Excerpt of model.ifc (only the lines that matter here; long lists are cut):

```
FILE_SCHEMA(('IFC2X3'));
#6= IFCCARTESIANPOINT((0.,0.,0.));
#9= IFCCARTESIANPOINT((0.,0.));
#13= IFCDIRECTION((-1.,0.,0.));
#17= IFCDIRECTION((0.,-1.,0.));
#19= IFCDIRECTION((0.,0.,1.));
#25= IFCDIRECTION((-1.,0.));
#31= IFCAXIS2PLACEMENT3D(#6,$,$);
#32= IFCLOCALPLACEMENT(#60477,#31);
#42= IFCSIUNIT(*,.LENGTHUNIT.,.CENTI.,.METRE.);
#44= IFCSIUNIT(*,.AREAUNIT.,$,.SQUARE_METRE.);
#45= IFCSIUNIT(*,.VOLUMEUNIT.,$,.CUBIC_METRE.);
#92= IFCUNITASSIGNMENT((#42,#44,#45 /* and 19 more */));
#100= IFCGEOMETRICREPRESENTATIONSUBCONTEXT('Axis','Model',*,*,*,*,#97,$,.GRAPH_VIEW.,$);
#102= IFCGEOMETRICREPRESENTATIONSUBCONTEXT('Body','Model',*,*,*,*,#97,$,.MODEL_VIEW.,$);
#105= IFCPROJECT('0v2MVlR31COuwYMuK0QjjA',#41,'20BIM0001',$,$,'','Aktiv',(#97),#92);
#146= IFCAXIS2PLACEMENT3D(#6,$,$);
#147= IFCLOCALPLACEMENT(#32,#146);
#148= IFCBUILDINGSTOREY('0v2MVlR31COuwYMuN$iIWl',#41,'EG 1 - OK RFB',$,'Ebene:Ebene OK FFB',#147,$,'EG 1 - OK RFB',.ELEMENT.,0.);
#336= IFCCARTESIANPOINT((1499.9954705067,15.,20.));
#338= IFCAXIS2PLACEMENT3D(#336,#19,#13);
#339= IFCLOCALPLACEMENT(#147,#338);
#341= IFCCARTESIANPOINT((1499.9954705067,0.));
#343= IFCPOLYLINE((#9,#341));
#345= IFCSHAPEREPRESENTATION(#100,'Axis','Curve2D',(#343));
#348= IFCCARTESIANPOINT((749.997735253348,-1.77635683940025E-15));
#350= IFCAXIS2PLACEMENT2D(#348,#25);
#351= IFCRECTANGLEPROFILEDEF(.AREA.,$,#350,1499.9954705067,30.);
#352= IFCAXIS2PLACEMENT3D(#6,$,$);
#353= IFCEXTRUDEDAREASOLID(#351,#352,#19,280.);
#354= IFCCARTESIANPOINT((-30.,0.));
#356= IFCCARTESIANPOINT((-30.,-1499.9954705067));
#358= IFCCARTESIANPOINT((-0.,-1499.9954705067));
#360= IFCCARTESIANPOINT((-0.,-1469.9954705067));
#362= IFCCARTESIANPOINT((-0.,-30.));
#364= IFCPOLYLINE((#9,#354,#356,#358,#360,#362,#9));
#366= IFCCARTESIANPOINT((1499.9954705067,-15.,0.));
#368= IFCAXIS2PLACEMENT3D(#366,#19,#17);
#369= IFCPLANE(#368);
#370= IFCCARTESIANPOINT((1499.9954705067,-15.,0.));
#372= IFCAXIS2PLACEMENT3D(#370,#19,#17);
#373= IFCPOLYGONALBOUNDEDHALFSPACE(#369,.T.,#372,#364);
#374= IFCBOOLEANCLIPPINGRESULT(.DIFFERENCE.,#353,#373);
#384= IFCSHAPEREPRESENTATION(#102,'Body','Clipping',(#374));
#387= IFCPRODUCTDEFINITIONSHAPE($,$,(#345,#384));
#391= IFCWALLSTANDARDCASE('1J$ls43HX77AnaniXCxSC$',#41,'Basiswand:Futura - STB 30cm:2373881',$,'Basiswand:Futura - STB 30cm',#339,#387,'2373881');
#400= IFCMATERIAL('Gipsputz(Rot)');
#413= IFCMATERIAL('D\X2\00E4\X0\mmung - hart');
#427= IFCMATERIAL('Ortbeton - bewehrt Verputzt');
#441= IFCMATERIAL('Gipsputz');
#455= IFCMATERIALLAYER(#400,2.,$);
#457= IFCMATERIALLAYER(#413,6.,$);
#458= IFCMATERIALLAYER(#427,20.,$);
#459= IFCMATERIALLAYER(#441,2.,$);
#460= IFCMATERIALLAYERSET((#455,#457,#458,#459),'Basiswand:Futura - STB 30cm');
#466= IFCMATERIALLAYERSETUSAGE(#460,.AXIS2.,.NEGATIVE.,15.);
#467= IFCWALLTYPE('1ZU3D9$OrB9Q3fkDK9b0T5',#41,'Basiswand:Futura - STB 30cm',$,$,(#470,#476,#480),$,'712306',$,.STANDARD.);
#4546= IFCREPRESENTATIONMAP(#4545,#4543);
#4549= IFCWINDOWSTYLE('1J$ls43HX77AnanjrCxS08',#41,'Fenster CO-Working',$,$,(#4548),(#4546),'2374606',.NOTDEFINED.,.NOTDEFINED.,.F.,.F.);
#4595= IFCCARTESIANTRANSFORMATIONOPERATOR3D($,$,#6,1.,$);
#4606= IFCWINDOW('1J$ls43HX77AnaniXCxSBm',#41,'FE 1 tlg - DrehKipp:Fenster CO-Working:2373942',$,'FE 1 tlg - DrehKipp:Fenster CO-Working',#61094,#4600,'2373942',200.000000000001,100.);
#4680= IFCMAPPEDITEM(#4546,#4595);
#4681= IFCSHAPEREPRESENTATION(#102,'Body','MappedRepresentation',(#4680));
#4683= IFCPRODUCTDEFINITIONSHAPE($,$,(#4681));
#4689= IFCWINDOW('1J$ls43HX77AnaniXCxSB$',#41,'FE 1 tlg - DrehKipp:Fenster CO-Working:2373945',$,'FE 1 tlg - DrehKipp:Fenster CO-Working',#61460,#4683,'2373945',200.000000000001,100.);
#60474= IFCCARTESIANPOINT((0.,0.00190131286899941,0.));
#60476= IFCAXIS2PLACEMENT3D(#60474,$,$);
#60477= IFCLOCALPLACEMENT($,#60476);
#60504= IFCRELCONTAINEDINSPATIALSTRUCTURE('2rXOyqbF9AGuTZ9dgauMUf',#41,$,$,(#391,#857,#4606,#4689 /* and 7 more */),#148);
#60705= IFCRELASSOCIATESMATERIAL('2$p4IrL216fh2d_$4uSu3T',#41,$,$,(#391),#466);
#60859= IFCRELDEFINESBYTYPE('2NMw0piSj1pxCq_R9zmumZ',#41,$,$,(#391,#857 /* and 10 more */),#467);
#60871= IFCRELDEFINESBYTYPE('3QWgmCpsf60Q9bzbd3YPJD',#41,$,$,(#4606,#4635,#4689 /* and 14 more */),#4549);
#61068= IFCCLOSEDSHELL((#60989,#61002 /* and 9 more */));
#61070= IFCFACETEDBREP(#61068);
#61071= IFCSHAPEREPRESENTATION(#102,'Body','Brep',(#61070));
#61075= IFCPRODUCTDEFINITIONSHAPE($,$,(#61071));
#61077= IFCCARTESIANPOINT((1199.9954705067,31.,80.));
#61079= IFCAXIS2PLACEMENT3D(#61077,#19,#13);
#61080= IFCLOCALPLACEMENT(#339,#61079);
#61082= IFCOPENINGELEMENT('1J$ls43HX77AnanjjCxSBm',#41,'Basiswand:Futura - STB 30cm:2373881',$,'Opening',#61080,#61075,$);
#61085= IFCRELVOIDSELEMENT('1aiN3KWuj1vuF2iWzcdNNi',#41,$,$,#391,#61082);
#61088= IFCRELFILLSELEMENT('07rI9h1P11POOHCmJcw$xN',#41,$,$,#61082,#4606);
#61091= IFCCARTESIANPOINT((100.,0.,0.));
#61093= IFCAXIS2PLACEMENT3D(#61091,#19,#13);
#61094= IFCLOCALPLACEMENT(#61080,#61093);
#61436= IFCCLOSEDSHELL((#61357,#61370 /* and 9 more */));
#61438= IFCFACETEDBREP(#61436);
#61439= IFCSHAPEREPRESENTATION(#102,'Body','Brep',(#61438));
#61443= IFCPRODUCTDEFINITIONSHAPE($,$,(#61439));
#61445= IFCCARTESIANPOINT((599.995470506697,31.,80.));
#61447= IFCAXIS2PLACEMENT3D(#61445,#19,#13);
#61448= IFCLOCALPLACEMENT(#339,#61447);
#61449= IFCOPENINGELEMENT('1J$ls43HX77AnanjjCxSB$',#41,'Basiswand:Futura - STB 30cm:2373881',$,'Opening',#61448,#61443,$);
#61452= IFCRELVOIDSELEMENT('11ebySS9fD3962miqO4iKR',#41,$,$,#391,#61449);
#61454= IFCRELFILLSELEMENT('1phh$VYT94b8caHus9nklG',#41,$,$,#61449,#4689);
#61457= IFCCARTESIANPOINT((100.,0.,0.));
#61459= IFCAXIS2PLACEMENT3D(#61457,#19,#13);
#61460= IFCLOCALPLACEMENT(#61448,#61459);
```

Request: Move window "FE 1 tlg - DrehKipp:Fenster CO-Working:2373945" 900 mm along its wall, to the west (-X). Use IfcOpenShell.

```python
import ifcopenshell
import ifcopenshell.api.geometry
import ifcopenshell.util.placement
import ifcopenshell.util.unit

model = ifcopenshell.open("model.ifc")
unit_scale = ifcopenshell.util.unit.calculate_unit_scale(model)

window = model.by_id(4689)
opening = window.FillsVoids[0].RelatingOpeningElement
wall = opening.VoidsElements[0].RelatingBuildingElement

wall_matrix = ifcopenshell.util.placement.get_local_placement(wall.ObjectPlacement)
shift = wall_matrix[:3, 0] * 0.9 / unit_scale
before = ifcopenshell.util.placement.get_local_placement(window.ObjectPlacement)[:3, 3].copy()

# The window is placed relative to its opening, so it follows when the opening moves.
matrix = ifcopenshell.util.placement.get_local_placement(opening.ObjectPlacement)
matrix[:3, 3] += shift
ifcopenshell.api.geometry.edit_object_placement(
    model, product=opening, matrix=matrix, is_si=False, should_transform_children=True
)

after = ifcopenshell.util.placement.get_local_placement(window.ObjectPlacement)[:3, 3]
print("window moved by", (after - before).round(3) + 0.0)

model.write("model_edited.ifc")
```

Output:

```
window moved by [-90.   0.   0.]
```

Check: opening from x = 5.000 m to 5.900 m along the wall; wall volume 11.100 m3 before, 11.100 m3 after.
